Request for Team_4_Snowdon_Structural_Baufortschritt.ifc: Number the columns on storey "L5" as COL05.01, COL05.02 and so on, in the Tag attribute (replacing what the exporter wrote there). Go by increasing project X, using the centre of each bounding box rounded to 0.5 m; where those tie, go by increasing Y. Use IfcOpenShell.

First a look at what the model holds.

```python
import ifcopenshell
import ifcopenshell.util.element
import ifcopenshell.util.placement

model = ifcopenshell.open("Team_4_Snowdon_Structural_Baufortschritt.ifc")
print(model.schema)
storey = next(s for s in model.by_type("IfcBuildingStorey") if s.Name == "L5")
columns = [e for e in ifcopenshell.util.element.get_decomposition(storey) if e.is_a("IfcColumn")]
for e in sorted(columns, key=lambda e: e.id()):
    origin = ifcopenshell.util.placement.get_local_placement(e.ObjectPlacement)[:3, 3]
    print(e.id(), e.Tag, e.Name, origin.round(2) + 0.0, sep=" | ")
```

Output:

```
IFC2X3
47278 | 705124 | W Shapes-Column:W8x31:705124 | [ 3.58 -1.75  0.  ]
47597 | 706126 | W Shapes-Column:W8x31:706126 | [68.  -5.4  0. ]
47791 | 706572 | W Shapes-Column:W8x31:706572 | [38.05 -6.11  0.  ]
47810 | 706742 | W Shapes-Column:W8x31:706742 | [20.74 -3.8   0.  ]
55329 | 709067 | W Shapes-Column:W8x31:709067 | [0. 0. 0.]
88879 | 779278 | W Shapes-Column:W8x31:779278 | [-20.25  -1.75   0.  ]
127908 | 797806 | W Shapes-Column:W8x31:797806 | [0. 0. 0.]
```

```python
import ifcopenshell
import ifcopenshell.geom
import ifcopenshell.util.element
import ifcopenshell.util.shape

model = ifcopenshell.open("Team_4_Snowdon_Structural_Baufortschritt.ifc")
settings = ifcopenshell.geom.settings()
settings.set("use-world-coords", True)


def centre(element):
    shape = ifcopenshell.geom.create_shape(settings, element)
    return ifcopenshell.util.shape.get_bbox_centroid(shape.geometry)


storey = next(s for s in model.by_type("IfcBuildingStorey") if s.Name == "L5")
columns = [e for e in ifcopenshell.util.element.get_decomposition(storey) if e.is_a("IfcColumn")]

# Insertion points can sit at a corner or the storey origin, so sort by the geometry (in metres).
centres = {e: centre(e) for e in columns}
columns.sort(key=lambda e: (round(centres[e][0] / 0.5), centres[e][1]))

for i, e in enumerate(columns, start=1):
    number = f"COL05.{i:02d}"
    e.Tag = number
    print(e.id(), number)

model.write("Team_4_Snowdon_Structural_Baufortschritt_v2.ifc")
```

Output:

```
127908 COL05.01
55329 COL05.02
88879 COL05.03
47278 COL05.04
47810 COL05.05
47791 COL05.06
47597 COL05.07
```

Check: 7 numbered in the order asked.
